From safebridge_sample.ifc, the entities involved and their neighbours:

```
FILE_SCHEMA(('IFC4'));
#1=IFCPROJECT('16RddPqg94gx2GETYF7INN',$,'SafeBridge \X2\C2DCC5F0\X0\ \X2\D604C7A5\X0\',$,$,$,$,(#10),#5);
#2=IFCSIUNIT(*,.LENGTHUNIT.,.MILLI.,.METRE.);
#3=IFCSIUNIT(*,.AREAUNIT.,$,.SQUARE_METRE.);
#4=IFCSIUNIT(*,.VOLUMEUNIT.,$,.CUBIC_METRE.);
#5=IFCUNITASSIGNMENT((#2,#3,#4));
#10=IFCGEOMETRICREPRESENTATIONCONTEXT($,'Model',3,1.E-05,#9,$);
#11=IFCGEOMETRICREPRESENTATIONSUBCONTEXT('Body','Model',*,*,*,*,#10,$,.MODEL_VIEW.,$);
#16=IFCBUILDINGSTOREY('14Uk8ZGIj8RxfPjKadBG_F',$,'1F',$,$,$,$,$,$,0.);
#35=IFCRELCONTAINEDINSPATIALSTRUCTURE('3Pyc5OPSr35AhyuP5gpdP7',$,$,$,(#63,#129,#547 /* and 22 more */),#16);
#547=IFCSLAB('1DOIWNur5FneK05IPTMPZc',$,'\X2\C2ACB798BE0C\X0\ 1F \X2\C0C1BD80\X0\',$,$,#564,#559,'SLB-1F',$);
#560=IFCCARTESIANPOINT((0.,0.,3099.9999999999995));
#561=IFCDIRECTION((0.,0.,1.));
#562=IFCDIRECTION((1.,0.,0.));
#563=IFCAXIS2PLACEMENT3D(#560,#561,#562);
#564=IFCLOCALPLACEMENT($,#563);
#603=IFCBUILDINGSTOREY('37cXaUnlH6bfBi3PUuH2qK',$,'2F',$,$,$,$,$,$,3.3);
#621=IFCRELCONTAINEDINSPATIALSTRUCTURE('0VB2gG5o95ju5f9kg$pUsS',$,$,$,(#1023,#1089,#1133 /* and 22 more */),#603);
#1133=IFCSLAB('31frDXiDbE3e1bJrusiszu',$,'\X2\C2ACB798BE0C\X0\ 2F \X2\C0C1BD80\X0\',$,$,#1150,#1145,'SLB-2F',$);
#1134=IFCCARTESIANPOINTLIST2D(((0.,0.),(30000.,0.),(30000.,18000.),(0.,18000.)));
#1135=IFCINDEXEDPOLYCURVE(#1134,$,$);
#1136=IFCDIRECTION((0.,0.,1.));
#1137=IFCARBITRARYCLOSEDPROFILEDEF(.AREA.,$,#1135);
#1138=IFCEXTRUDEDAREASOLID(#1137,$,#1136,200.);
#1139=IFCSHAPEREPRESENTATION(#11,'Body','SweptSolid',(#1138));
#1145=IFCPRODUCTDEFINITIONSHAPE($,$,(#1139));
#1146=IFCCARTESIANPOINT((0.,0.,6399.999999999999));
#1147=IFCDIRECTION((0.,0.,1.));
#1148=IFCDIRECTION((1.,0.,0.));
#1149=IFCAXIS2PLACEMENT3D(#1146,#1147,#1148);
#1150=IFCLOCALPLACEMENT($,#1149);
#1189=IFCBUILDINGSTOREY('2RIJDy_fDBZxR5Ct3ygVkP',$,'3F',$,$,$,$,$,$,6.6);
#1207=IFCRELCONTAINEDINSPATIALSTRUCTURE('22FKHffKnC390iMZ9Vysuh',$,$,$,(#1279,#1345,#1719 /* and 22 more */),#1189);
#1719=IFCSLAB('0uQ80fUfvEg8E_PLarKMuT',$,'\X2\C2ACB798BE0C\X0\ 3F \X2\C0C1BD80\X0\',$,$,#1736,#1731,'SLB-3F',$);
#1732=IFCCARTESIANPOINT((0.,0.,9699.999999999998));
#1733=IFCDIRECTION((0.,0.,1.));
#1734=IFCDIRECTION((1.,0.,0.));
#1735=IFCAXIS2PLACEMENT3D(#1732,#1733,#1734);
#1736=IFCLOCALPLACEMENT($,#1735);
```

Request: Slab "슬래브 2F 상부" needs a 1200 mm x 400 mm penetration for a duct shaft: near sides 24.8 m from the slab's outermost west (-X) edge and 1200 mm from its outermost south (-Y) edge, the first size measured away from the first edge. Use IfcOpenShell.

```python
import numpy as np
import ifcopenshell
import ifcopenshell.api.feature
import ifcopenshell.api.geometry
import ifcopenshell.api.root
import ifcopenshell.geom
import ifcopenshell.util.placement
import ifcopenshell.util.representation
import ifcopenshell.util.shape
import ifcopenshell.util.unit

model = ifcopenshell.open("safebridge_sample.ifc")
unit_scale = ifcopenshell.util.unit.calculate_unit_scale(model)
settings = ifcopenshell.geom.settings()


def volume(element):
    """Net volume in cubic metres, openings subtracted."""
    shape = ifcopenshell.geom.create_shape(settings, element)
    return ifcopenshell.util.shape.get_volume(shape.geometry)


slab = model.by_guid("31frDXiDbE3e1bJrusiszu")
before = volume(slab)

# Extent in the slab's own axes, in metres. The edges named are its -X and -Y sides.
slab_shape = ifcopenshell.geom.create_shape(settings, slab)
vertices = ifcopenshell.util.shape.get_vertices(slab_shape.geometry)
x_min, y_min, bottom = vertices.min(axis=0)
top = vertices[:, 2].max()

opening = ifcopenshell.api.root.create_entity(model, ifc_class="IfcOpeningElement", name="Duct shaft opening", predefined_type="OPENING")
context = ifcopenshell.util.representation.get_context(model, "Model", "Body", "MODEL_VIEW")
width, depth = 1.2, 0.4
outline = [(0.0, 0.0), (width, 0.0), (width, depth), (0.0, depth), (0.0, 0.0)]
# Overshoot both faces by 50 mm so the cut is clean.
shape = ifcopenshell.api.geometry.add_slab_representation(
    model, context=context, depth=top - bottom + 0.1, polyline=outline
)
ifcopenshell.api.geometry.assign_representation(model, product=opening, representation=shape)

matrix = ifcopenshell.util.placement.get_local_placement(slab.ObjectPlacement)
matrix[:, 3] = matrix @ np.append(np.array([x_min + 24.8, y_min + 1.2, bottom - 0.05]) / unit_scale, 1.0)
ifcopenshell.api.geometry.edit_object_placement(model, product=opening, matrix=matrix, is_si=False)
ifcopenshell.api.feature.add_feature(model, feature=opening, element=slab)

after = volume(slab)

print(f"slab volume {before:.3f} -> {after:.3f} m3")

model.write("safebridge_sample_rev.ifc")
```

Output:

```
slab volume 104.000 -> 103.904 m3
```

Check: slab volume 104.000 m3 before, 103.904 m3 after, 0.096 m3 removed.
